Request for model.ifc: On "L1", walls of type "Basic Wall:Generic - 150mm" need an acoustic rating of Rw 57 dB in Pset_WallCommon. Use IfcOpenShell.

First a look at what the model holds.

```python
import ifcopenshell
import ifcopenshell.util.element

model = ifcopenshell.open("model.ifc")
print(model.schema)
storey = next(s for s in model.by_type("IfcBuildingStorey") if s.Name == "L1")
walls = [e for e in ifcopenshell.util.element.get_decomposition(storey) if e.is_a("IfcWall")]
seen = {}
for e in walls:
    element_type = ifcopenshell.util.element.get_type(e)
    key = (element_type.Name if element_type != e and element_type else None, ifcopenshell.util.element.get_pset(e, "Pset_WallCommon", "AcousticRating"))
    seen[key] = seen.get(key, 0) + 1
for (name, value), count in sorted(seen.items(), key=str):
    print(count, "x", name, "|", value)
```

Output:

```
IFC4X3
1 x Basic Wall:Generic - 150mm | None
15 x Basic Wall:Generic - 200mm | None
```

```python
import ifcopenshell
import ifcopenshell.api.pset
import ifcopenshell.util.element

model = ifcopenshell.open("model.ifc")

storey = next(s for s in model.by_type("IfcBuildingStorey") if s.Name == "L1")
walls = [e for e in ifcopenshell.util.element.get_decomposition(storey) if e.is_a("IfcWall")]

count = 0
for e in walls:
    element_type = ifcopenshell.util.element.get_type(e)
    if element_type in (None, e) or element_type.Name != "Basic Wall:Generic - 150mm":
        continue
    # add_pset returns the element's existing set when there is one.
    pset = ifcopenshell.api.pset.add_pset(model, product=e, name="Pset_WallCommon")
    ifcopenshell.api.pset.edit_pset(model, pset=pset, properties={"AcousticRating": "Rw 57 dB"})
    count += 1

print(count, "walls updated")

model.write("model_v2.ifc")
```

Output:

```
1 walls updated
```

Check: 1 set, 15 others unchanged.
